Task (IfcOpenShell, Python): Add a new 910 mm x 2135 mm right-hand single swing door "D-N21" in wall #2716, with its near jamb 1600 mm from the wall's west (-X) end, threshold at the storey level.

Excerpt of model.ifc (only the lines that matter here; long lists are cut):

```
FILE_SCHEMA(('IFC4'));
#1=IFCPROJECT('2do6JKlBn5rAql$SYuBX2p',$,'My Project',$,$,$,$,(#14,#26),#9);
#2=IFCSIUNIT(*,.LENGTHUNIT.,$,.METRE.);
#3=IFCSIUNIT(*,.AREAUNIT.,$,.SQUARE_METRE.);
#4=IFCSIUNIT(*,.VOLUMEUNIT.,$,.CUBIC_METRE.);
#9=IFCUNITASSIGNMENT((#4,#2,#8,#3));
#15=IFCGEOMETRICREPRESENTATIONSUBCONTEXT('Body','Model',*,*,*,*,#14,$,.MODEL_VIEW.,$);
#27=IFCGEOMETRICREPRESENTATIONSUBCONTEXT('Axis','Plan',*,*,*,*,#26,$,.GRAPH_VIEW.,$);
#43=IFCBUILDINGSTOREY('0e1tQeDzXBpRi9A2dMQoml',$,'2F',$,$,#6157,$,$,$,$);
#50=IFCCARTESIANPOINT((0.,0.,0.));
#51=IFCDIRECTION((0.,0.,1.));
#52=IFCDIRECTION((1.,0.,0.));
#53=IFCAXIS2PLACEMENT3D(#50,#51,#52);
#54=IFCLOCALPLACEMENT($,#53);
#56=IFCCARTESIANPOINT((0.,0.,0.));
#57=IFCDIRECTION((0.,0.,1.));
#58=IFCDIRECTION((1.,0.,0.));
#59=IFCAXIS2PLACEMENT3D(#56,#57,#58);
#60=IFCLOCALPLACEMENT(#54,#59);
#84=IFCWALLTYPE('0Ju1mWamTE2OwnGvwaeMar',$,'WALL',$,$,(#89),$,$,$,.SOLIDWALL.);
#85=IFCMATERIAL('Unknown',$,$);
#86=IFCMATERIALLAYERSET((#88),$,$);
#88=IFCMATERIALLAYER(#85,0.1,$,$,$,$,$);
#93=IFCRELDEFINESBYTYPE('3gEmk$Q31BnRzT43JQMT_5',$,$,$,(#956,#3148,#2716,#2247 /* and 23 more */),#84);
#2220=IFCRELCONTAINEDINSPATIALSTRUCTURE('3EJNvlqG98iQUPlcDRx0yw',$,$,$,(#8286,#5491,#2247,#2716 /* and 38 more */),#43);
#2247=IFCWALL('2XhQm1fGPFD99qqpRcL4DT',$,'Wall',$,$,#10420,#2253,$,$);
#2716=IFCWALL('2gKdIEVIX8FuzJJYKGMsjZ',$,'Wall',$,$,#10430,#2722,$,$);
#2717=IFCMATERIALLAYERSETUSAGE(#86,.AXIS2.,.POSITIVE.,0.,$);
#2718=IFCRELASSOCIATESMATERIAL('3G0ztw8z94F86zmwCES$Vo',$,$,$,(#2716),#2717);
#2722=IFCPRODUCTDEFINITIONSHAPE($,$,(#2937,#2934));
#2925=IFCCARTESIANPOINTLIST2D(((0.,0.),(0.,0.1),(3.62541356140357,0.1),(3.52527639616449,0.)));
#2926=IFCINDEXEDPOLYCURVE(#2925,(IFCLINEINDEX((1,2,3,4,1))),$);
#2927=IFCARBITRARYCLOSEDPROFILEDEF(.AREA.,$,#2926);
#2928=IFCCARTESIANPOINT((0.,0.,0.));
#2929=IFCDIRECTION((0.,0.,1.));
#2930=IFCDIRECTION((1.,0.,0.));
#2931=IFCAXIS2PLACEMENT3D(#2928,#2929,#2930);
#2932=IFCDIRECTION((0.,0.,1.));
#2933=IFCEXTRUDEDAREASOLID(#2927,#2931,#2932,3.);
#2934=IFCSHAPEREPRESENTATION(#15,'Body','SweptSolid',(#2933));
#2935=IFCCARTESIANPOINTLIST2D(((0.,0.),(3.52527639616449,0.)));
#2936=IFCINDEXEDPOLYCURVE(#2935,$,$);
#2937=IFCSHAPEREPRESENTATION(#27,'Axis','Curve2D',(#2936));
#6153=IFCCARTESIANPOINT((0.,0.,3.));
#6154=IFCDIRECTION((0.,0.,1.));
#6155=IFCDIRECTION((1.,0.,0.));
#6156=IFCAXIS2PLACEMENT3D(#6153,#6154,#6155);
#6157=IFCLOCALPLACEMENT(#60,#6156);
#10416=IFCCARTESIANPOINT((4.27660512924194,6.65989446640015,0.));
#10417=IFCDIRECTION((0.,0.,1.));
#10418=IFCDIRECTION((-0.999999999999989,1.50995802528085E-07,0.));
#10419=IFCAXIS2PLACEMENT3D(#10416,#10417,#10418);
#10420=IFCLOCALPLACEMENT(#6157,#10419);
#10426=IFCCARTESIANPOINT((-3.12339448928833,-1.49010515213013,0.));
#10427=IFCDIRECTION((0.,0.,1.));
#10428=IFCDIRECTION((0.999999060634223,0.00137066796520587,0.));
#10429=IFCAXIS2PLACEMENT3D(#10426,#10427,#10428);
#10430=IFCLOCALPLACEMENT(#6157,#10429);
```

```python
import numpy as np
import ifcopenshell
import ifcopenshell.api.feature
import ifcopenshell.api.geometry
import ifcopenshell.api.root
import ifcopenshell.api.spatial
import ifcopenshell.geom
import ifcopenshell.util.element
import ifcopenshell.util.placement
import ifcopenshell.util.representation
import ifcopenshell.util.shape
import ifcopenshell.util.unit

model = ifcopenshell.open("model.ifc")
unit_scale = ifcopenshell.util.unit.calculate_unit_scale(model)
settings = ifcopenshell.geom.settings()


def volume(element):
    """Net volume in cubic metres, openings subtracted."""
    shape = ifcopenshell.geom.create_shape(settings, element)
    return ifcopenshell.util.shape.get_volume(shape.geometry)


wall = model.by_guid("2gKdIEVIX8FuzJJYKGMsjZ")
storey = ifcopenshell.util.element.get_container(wall, ifc_class="IfcBuildingStorey")
context = ifcopenshell.util.representation.get_context(model, "Model", "Body", "MODEL_VIEW")
before = volume(wall)

width, height, from_end, sill = 0.91, 2.135, 1.6, 0.0  # metres

# The wall runs along its own X axis, and the end named is its -X end.
wall_shape = ifcopenshell.geom.create_shape(settings, wall)
x, y, z = ifcopenshell.util.shape.get_vertices(wall_shape.geometry).T
start = x.min() + from_end
face, thickness = float(y.min()), float(y.max() - y.min())
wall_matrix = ifcopenshell.util.placement.get_local_placement(wall.ObjectPlacement)
level = ifcopenshell.util.placement.get_local_placement(storey.ObjectPlacement)[2, 3]


def in_wall(x, y):
    """Placement at x, y metres in the wall's axes, at sill height."""
    matrix = wall_matrix.copy()
    matrix[:, 3] = wall_matrix @ np.array([x / unit_scale, y / unit_scale, 0.0, 1.0])
    matrix[2, 3] = level + sill / unit_scale
    return matrix


# Opening: a box that overshoots both wall faces by 50 mm.
opening = ifcopenshell.api.root.create_entity(model, ifc_class="IfcOpeningElement", predefined_type="OPENING")
box = ifcopenshell.api.geometry.add_wall_representation(
    model, context=context, length=width, height=height, thickness=thickness + 0.1
)
ifcopenshell.api.geometry.assign_representation(model, product=opening, representation=box)
ifcopenshell.api.geometry.edit_object_placement(model, product=opening, matrix=in_wall(start, face - 0.05), is_si=False)
ifcopenshell.api.feature.add_feature(model, feature=opening, element=wall)

door = ifcopenshell.api.root.create_entity(model, ifc_class="IfcDoor", name="D-N21", predefined_type="DOOR")
door.OverallWidth, door.OverallHeight = width / unit_scale, height / unit_scale
door.OperationType = "SINGLE_SWING_RIGHT"
body = ifcopenshell.api.geometry.add_door_representation(
    model,
    context=context,
    overall_width=door.OverallWidth,
    overall_height=door.OverallHeight,
    operation_type="SINGLE_SWING_RIGHT",
    lining_properties={"LiningDepth": thickness / unit_scale, "ThresholdDepth": thickness / unit_scale},
)
ifcopenshell.api.geometry.assign_representation(model, product=door, representation=body)
ifcopenshell.api.spatial.assign_container(model, products=[door], relating_structure=storey)
ifcopenshell.api.feature.add_filling(model, opening=opening, element=door)

# The lining spans the wall, so the door starts at the wall face.
ifcopenshell.api.geometry.edit_object_placement(model, product=door, matrix=in_wall(start, face), is_si=False)

after = volume(wall)

print(f"wall volume {before:.3f} -> {after:.3f} m3")

model.write("model_v2.ifc")
```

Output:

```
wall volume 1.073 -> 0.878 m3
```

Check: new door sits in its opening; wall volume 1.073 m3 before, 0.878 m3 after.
